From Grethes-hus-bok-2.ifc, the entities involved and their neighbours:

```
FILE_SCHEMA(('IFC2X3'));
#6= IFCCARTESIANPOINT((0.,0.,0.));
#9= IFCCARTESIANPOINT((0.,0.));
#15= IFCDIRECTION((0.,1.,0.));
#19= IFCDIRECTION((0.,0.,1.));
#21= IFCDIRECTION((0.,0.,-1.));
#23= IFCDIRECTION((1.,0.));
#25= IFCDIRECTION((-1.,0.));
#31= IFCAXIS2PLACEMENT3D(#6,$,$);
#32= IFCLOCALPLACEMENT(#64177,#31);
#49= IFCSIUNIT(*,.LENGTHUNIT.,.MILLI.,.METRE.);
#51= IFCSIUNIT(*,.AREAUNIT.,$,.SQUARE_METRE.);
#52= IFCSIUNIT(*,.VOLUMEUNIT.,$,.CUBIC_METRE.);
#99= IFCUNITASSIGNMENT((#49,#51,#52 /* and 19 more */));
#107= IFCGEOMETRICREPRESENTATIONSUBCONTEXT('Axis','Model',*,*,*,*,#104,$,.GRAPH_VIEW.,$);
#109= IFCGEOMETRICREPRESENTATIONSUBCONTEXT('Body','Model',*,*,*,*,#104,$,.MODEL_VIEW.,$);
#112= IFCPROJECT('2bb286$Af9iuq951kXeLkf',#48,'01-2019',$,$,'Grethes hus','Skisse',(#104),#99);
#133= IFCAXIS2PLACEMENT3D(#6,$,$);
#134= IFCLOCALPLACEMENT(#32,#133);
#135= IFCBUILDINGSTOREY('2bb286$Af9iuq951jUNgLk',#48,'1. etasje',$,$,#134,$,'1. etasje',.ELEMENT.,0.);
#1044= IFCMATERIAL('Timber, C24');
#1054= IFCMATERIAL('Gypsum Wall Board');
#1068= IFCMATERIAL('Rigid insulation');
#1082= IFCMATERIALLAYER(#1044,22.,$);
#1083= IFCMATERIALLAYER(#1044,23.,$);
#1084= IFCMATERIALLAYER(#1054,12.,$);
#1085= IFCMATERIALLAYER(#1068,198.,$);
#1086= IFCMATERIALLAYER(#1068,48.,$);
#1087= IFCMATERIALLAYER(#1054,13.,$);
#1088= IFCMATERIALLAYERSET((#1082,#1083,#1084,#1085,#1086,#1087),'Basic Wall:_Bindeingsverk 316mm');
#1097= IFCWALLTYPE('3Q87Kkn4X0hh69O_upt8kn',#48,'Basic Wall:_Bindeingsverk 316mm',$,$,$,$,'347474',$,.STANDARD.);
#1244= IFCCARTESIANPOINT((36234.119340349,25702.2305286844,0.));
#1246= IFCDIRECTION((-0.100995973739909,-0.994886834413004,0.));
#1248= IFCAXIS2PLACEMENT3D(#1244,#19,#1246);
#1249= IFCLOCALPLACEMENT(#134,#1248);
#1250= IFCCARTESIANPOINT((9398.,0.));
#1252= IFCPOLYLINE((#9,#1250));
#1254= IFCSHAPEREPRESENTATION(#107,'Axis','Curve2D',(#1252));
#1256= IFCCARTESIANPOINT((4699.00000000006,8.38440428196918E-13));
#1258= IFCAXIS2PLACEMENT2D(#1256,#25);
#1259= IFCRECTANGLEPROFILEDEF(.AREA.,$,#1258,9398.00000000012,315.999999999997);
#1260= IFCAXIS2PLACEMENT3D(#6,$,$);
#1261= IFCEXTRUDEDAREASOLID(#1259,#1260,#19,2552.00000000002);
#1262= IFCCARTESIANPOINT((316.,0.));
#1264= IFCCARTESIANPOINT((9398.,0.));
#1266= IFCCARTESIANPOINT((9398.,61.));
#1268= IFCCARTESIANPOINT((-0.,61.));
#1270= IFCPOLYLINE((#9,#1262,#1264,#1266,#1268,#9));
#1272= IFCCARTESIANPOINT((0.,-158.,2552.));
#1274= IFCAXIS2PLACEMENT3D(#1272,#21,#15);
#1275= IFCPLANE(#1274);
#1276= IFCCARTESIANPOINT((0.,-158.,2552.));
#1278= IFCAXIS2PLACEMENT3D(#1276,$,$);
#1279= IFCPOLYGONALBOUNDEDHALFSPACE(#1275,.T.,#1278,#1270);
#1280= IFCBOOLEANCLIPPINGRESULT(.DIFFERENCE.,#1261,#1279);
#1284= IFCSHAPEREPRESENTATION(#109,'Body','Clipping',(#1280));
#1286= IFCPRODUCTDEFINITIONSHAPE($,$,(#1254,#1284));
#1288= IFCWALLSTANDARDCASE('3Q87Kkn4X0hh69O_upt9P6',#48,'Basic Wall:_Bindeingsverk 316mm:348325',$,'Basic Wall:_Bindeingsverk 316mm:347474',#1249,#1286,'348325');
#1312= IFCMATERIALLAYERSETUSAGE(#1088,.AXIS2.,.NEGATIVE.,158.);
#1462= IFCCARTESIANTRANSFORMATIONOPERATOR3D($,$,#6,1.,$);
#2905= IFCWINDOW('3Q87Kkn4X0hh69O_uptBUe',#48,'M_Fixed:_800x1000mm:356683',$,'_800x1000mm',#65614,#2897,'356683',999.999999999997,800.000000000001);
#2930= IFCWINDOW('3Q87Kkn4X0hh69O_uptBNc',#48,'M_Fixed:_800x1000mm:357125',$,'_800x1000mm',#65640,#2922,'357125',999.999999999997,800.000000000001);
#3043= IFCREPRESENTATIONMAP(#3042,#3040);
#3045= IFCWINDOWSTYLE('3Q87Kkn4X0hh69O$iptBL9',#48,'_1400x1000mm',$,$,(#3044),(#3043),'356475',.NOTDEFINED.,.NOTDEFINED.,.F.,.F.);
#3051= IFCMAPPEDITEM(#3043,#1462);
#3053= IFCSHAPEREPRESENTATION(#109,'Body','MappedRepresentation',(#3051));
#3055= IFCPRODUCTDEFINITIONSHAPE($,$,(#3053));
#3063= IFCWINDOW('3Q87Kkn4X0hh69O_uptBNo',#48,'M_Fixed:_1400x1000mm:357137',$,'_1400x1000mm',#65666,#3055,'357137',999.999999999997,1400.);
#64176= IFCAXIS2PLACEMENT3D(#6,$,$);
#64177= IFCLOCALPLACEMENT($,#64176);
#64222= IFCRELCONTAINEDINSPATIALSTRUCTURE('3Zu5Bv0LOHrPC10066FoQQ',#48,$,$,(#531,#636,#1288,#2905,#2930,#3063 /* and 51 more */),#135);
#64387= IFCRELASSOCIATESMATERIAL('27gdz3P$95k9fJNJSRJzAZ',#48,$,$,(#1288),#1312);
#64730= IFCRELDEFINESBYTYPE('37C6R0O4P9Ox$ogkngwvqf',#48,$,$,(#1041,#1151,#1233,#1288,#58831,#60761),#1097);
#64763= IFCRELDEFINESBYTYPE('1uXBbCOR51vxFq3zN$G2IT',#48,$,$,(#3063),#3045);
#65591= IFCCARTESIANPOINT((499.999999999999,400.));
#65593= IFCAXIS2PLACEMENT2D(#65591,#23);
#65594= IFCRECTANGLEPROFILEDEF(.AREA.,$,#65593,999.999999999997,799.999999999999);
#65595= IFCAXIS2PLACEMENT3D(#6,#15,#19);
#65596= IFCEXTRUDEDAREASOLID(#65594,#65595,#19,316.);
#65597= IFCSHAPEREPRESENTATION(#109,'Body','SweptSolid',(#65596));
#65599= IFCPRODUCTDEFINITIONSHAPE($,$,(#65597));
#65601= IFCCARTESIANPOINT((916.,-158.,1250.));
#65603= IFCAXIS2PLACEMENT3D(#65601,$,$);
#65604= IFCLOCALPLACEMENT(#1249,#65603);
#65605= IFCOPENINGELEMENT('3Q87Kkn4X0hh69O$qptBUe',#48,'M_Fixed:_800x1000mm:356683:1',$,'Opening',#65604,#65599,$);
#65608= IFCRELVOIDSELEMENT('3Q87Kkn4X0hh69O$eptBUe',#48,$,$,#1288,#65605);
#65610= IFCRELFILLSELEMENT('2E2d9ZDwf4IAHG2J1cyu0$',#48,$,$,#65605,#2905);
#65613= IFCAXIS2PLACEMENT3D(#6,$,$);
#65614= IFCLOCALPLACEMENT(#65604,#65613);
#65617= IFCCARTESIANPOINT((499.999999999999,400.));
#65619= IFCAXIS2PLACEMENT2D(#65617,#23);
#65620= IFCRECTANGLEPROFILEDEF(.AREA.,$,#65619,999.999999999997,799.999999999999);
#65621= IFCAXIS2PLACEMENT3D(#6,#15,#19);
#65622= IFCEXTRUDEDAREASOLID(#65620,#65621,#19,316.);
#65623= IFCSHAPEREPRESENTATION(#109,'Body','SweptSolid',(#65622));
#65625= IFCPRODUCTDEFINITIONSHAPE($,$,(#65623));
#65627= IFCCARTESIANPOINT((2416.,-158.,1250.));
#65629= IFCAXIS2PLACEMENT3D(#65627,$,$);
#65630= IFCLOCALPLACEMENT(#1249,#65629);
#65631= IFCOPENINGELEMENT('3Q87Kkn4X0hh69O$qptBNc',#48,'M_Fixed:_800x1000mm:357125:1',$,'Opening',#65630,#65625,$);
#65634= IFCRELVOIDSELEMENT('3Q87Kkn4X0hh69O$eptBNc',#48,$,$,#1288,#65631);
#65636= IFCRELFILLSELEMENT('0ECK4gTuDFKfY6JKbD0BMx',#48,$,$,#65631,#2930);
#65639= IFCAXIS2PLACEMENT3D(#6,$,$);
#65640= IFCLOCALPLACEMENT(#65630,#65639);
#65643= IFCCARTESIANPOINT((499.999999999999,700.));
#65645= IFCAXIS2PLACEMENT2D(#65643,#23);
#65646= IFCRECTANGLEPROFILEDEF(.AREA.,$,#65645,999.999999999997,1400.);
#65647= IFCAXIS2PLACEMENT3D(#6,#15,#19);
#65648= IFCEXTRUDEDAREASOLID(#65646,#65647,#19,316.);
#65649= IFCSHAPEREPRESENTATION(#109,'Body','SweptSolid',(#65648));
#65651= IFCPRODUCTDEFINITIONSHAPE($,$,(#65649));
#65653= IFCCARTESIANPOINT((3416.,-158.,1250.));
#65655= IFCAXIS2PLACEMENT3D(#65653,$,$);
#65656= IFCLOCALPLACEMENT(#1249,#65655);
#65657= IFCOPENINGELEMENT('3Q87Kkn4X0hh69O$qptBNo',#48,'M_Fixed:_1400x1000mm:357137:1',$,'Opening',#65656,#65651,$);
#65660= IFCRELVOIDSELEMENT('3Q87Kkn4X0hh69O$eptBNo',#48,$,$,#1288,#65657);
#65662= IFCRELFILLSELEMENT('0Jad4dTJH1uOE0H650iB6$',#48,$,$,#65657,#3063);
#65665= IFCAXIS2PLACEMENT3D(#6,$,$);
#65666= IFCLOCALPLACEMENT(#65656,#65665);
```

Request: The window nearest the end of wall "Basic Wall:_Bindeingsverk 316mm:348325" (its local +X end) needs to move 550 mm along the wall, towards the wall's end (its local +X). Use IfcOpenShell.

```python
import ifcopenshell
import ifcopenshell.api.geometry
import ifcopenshell.util.placement
import ifcopenshell.util.unit

model = ifcopenshell.open("Grethes-hus-bok-2.ifc")
unit_scale = ifcopenshell.util.unit.calculate_unit_scale(model)

window = model.by_id(3063)
opening = window.FillsVoids[0].RelatingOpeningElement
wall = opening.VoidsElements[0].RelatingBuildingElement

wall_matrix = ifcopenshell.util.placement.get_local_placement(wall.ObjectPlacement)
shift = wall_matrix[:3, 0] * 0.55 / unit_scale
before = ifcopenshell.util.placement.get_local_placement(window.ObjectPlacement)[:3, 3].copy()

# The window is placed relative to its opening, so it follows when the opening moves.
matrix = ifcopenshell.util.placement.get_local_placement(opening.ObjectPlacement)
matrix[:3, 3] += shift
ifcopenshell.api.geometry.edit_object_placement(
    model, product=opening, matrix=matrix, is_si=False, should_transform_children=True
)

after = ifcopenshell.util.placement.get_local_placement(window.ObjectPlacement)[:3, 3]
print("window moved by", (after - before).round(3) + 0.0)

model.write("Grethes-hus-bok-2_v2.ifc")
```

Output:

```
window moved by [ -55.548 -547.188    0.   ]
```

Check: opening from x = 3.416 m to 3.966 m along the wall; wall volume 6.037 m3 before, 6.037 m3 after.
